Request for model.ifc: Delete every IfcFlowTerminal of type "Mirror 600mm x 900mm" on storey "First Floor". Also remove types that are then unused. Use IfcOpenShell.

First a look at what the model holds.

```python
import ifcopenshell
import ifcopenshell.util.element

model = ifcopenshell.open("model.ifc")
print(model.schema)
storey = next(s for s in model.by_type("IfcBuildingStorey") if s.Name == "First Floor")
terminals = [e for e in ifcopenshell.util.element.get_decomposition(storey) if e.is_a("IfcFlowTerminal")]
seen = {}
for e in terminals:
    element_type = ifcopenshell.util.element.get_type(e)
    name = element_type.Name if element_type not in (None, e) else None
    seen[name] = seen.get(name, 0) + 1
for name, count in sorted(seen.items(), key=str):
    print(count, "x", name)
```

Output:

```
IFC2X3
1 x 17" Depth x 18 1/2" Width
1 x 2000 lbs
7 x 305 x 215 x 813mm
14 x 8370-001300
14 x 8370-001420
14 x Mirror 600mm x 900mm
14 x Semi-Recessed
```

```python
import ifcopenshell
import ifcopenshell.api.root
import ifcopenshell.util.element

model = ifcopenshell.open("model.ifc")

storey = next(s for s in model.by_type("IfcBuildingStorey") if s.Name == "First Floor")
terminals = [e for e in ifcopenshell.util.element.get_decomposition(storey) if e.is_a("IfcFlowTerminal")]
targets = [e for e in terminals if (t := ifcopenshell.util.element.get_type(e)) not in (None, e) and t.Name == "Mirror 600mm x 900mm"]
types = {ifcopenshell.util.element.get_type(e) for e in targets} - {None, *targets}

for e in targets:
    ifcopenshell.api.root.remove_product(model, product=e)
print(len(targets), "removed")

unused = [t for t in types if not ifcopenshell.util.element.get_types(t)]
for t in unused:
    ifcopenshell.api.root.remove_product(model, product=t)
print(len(unused), "unused types removed")

model.write("model_rev.ifc")
```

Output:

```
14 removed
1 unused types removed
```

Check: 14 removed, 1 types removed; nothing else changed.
